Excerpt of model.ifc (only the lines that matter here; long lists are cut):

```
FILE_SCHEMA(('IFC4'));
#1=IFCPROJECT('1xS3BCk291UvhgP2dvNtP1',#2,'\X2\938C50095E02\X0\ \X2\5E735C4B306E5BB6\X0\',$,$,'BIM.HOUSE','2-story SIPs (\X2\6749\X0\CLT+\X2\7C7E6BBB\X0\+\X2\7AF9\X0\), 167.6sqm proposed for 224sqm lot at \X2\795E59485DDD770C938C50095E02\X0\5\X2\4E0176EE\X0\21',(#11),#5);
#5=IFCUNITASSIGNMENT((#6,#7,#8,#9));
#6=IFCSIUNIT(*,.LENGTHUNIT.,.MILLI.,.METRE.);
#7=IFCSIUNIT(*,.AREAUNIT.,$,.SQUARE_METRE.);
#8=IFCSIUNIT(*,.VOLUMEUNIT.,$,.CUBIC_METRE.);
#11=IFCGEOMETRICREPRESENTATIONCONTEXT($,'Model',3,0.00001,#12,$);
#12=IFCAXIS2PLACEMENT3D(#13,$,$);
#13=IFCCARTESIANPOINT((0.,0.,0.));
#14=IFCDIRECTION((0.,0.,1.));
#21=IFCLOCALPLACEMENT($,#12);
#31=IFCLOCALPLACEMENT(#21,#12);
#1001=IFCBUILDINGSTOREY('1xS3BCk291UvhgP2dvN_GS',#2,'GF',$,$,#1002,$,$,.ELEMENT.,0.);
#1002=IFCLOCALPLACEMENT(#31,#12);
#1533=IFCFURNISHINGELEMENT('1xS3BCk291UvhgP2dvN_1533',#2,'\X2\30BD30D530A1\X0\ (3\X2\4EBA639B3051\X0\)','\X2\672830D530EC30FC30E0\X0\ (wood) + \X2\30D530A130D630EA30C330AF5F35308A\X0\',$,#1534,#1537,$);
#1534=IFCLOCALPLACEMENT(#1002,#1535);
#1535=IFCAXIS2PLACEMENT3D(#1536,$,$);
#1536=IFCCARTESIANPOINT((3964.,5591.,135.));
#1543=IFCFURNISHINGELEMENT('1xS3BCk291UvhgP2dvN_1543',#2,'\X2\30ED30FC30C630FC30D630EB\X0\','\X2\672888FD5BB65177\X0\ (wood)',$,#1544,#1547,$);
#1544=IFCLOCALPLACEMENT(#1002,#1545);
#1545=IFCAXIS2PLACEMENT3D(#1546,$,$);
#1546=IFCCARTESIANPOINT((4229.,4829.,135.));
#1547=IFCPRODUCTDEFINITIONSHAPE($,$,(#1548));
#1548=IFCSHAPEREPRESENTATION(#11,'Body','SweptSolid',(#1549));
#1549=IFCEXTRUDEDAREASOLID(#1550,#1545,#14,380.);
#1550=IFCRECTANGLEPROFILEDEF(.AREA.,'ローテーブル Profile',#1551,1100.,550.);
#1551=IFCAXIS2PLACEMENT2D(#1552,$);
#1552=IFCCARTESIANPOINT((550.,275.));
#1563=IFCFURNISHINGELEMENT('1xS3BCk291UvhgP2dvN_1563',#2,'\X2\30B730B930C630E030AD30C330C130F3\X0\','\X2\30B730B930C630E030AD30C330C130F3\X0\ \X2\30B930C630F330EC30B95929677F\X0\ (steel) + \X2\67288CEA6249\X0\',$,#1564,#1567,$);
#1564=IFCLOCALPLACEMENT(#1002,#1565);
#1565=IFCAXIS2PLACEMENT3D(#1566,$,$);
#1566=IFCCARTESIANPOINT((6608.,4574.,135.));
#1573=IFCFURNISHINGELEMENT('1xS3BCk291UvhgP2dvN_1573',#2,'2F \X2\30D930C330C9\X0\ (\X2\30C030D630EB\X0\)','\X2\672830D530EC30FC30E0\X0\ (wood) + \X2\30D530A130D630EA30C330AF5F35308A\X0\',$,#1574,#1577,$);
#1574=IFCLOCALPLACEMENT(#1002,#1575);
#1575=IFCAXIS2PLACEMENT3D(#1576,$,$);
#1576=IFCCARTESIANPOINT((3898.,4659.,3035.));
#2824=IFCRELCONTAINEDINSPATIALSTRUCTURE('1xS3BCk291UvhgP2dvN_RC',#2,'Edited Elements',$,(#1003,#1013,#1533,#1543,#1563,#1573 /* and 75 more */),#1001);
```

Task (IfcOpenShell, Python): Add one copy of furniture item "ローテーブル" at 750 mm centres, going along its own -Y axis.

```python
import ifcopenshell
import ifcopenshell.api.geometry
import ifcopenshell.api.root
import ifcopenshell.util.element
import ifcopenshell.util.placement
import ifcopenshell.util.unit

model = ifcopenshell.open("model.ifc")
unit_scale = ifcopenshell.util.unit.calculate_unit_scale(model)


def reuse_history(source, copy):
    """copy_class also copies each property set's owner history, people and application; keep the originals."""
    for rel in copy.IsDefinedBy:
        if rel.is_a("IfcRelDefinesByProperties") and (history := rel.RelatingPropertyDefinition.OwnerHistory):
            rel.RelatingPropertyDefinition.OwnerHistory = source.OwnerHistory
            ifcopenshell.util.element.remove_deep2(model, history)


source = model.by_guid("1xS3BCk291UvhgP2dvN_1543")
base = ifcopenshell.util.placement.get_local_placement(source.ObjectPlacement)
step = -base[:3, 1] * 0.75 / unit_scale

for i in range(1, 2):
    copy = ifcopenshell.api.root.copy_class(model, product=source)
    copy.Representation = ifcopenshell.util.element.copy_deep(
        model, source.Representation, exclude=["IfcGeometricRepresentationContext", "IfcRepresentationMap"]
    )
    reuse_history(source, copy)
    matrix = base.copy()
    matrix[:3, 3] += i * step
    print("added at", matrix[:3, 3].round(3) + 0.0)
    ifcopenshell.api.geometry.edit_object_placement(model, product=copy, matrix=matrix, is_si=False)

model.write("model_updated.ifc")
```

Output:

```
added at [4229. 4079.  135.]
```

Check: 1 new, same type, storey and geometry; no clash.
